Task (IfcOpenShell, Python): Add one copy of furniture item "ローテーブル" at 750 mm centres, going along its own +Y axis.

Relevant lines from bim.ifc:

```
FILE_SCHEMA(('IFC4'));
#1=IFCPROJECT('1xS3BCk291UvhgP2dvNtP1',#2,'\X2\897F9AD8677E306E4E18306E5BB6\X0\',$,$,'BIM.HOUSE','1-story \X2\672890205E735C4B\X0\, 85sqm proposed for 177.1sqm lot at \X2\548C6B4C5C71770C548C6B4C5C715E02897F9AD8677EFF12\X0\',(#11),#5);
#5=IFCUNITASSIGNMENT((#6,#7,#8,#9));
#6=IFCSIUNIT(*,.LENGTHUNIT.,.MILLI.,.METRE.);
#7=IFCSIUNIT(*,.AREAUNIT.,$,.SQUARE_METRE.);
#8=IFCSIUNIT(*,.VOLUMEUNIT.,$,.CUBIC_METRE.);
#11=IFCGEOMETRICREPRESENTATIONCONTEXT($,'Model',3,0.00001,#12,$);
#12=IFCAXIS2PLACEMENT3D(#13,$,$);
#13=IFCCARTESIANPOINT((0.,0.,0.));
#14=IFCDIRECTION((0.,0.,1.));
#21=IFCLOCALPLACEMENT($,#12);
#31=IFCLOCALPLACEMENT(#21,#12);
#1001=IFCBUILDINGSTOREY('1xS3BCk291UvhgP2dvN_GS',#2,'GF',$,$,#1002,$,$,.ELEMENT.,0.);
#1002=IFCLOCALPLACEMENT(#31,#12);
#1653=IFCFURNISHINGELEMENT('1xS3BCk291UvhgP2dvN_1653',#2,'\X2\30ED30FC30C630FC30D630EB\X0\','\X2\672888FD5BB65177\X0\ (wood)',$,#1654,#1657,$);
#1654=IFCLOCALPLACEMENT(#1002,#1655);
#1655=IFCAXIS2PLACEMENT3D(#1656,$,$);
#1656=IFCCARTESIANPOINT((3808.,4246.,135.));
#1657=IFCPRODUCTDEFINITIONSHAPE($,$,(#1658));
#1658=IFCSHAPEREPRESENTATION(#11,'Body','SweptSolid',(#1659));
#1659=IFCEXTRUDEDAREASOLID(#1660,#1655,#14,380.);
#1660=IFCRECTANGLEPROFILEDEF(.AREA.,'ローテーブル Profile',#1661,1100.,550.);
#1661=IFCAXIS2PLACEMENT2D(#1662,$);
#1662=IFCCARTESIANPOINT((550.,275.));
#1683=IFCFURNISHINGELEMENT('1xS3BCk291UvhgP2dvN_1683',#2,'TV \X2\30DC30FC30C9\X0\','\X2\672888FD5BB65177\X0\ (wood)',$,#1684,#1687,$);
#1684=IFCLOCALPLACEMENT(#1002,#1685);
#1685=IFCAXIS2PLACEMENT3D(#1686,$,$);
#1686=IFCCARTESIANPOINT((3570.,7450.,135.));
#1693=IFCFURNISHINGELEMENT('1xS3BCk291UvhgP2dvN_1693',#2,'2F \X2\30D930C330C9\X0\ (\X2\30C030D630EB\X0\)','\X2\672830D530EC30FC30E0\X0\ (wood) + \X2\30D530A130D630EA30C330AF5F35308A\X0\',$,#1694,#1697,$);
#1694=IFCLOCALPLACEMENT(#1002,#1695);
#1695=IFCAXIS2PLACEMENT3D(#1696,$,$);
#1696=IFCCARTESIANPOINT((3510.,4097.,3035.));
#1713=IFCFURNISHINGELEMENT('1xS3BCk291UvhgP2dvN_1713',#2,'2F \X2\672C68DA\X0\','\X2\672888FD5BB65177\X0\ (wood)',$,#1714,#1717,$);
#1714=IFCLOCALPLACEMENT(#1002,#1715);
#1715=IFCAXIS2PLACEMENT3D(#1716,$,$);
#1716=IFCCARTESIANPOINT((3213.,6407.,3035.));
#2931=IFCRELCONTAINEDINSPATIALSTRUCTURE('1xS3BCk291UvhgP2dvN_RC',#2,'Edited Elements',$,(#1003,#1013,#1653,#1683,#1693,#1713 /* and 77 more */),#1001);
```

```python
import ifcopenshell
import ifcopenshell.api.geometry
import ifcopenshell.api.root
import ifcopenshell.util.element
import ifcopenshell.util.placement

model = ifcopenshell.open("bim.ifc")


def reuse_history(source, copy):
    """copy_class also copies each property set's owner history, people and application; keep the originals."""
    for rel in copy.IsDefinedBy:
        if rel.is_a("IfcRelDefinesByProperties") and (history := rel.RelatingPropertyDefinition.OwnerHistory):
            rel.RelatingPropertyDefinition.OwnerHistory = source.OwnerHistory
            ifcopenshell.util.element.remove_deep2(model, history)


source = model.by_id(1653)
base = ifcopenshell.util.placement.get_local_placement(source.ObjectPlacement)
step = base[:3, 1] * 750.0

for i in range(1, 2):
    copy = ifcopenshell.api.root.copy_class(model, product=source)
    copy.Representation = ifcopenshell.util.element.copy_deep(
        model, source.Representation, exclude=["IfcGeometricRepresentationContext", "IfcRepresentationMap"]
    )
    reuse_history(source, copy)
    matrix = base.copy()
    matrix[:3, 3] += i * step
    print("added at", matrix[:3, 3].round(3) + 0.0)
    ifcopenshell.api.geometry.edit_object_placement(model, product=copy, matrix=matrix, is_si=False)

model.write("bim_v2.ifc")
```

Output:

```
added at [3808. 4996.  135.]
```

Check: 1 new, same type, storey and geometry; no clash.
